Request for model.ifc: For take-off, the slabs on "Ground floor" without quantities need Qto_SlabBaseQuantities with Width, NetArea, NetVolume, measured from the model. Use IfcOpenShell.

First a look at what the model holds.

```python
import ifcopenshell
import ifcopenshell.util.element
import ifcopenshell.util.unit

model = ifcopenshell.open("model.ifc")
print(model.schema)
for unit_type in ("LENGTHUNIT", "AREAUNIT", "VOLUMEUNIT"):
    print(unit_type, ifcopenshell.util.unit.calculate_unit_scale(model, unit_type))
storey = next(s for s in model.by_type("IfcBuildingStorey") if s.Name == "Ground floor")
slabs = [e for e in ifcopenshell.util.element.get_decomposition(storey) if e.is_a("IfcSlab")]
for e in sorted(slabs, key=lambda e: e.id()):
    print(e.id(), e.is_a(), e.Name, list(ifcopenshell.util.element.get_psets(e, qtos_only=True)), sep=" | ")
```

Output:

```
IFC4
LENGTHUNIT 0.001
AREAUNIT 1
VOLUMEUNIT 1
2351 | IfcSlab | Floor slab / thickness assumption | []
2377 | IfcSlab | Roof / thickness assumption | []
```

```python
import ifcopenshell
import ifcopenshell.api.pset
import ifcopenshell.geom
import ifcopenshell.util.element
import ifcopenshell.util.shape
import ifcopenshell.util.unit

model = ifcopenshell.open("model.ifc")
unit_scale = ifcopenshell.util.unit.calculate_unit_scale(model)
area_scale = ifcopenshell.util.unit.calculate_unit_scale(model, "AREAUNIT")
volume_scale = ifcopenshell.util.unit.calculate_unit_scale(model, "VOLUMEUNIT")
settings = ifcopenshell.geom.settings()

storey = next(s for s in model.by_type("IfcBuildingStorey") if s.Name == "Ground floor")
slabs = [e for e in ifcopenshell.util.element.get_decomposition(storey) if e.is_a("IfcSlab")]

for e in sorted(slabs, key=lambda e: e.id()):
    if ifcopenshell.util.element.get_psets(e, qtos_only=True, should_inherit=False):
        continue
    # Geometry comes back in metres, in the element's own axes.
    shape = ifcopenshell.geom.create_shape(settings, e)
    values = {
        "Width": ifcopenshell.util.shape.get_z(shape.geometry) / unit_scale,
        "NetArea": ifcopenshell.util.shape.get_footprint_area(shape.geometry) / area_scale,
        "NetVolume": ifcopenshell.util.shape.get_volume(shape.geometry) / volume_scale,
    }
    qto = ifcopenshell.api.pset.add_qto(model, product=e, name="Qto_SlabBaseQuantities")
    ifcopenshell.api.pset.edit_qto(model, qto=qto, properties=values)
    print(e.id(), {k: round(v, 3) for k, v in values.items()})

model.write("model_rev.ifc")
```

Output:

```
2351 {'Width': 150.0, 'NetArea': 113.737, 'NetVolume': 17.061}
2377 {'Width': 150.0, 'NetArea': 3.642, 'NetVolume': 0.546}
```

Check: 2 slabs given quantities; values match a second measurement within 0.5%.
